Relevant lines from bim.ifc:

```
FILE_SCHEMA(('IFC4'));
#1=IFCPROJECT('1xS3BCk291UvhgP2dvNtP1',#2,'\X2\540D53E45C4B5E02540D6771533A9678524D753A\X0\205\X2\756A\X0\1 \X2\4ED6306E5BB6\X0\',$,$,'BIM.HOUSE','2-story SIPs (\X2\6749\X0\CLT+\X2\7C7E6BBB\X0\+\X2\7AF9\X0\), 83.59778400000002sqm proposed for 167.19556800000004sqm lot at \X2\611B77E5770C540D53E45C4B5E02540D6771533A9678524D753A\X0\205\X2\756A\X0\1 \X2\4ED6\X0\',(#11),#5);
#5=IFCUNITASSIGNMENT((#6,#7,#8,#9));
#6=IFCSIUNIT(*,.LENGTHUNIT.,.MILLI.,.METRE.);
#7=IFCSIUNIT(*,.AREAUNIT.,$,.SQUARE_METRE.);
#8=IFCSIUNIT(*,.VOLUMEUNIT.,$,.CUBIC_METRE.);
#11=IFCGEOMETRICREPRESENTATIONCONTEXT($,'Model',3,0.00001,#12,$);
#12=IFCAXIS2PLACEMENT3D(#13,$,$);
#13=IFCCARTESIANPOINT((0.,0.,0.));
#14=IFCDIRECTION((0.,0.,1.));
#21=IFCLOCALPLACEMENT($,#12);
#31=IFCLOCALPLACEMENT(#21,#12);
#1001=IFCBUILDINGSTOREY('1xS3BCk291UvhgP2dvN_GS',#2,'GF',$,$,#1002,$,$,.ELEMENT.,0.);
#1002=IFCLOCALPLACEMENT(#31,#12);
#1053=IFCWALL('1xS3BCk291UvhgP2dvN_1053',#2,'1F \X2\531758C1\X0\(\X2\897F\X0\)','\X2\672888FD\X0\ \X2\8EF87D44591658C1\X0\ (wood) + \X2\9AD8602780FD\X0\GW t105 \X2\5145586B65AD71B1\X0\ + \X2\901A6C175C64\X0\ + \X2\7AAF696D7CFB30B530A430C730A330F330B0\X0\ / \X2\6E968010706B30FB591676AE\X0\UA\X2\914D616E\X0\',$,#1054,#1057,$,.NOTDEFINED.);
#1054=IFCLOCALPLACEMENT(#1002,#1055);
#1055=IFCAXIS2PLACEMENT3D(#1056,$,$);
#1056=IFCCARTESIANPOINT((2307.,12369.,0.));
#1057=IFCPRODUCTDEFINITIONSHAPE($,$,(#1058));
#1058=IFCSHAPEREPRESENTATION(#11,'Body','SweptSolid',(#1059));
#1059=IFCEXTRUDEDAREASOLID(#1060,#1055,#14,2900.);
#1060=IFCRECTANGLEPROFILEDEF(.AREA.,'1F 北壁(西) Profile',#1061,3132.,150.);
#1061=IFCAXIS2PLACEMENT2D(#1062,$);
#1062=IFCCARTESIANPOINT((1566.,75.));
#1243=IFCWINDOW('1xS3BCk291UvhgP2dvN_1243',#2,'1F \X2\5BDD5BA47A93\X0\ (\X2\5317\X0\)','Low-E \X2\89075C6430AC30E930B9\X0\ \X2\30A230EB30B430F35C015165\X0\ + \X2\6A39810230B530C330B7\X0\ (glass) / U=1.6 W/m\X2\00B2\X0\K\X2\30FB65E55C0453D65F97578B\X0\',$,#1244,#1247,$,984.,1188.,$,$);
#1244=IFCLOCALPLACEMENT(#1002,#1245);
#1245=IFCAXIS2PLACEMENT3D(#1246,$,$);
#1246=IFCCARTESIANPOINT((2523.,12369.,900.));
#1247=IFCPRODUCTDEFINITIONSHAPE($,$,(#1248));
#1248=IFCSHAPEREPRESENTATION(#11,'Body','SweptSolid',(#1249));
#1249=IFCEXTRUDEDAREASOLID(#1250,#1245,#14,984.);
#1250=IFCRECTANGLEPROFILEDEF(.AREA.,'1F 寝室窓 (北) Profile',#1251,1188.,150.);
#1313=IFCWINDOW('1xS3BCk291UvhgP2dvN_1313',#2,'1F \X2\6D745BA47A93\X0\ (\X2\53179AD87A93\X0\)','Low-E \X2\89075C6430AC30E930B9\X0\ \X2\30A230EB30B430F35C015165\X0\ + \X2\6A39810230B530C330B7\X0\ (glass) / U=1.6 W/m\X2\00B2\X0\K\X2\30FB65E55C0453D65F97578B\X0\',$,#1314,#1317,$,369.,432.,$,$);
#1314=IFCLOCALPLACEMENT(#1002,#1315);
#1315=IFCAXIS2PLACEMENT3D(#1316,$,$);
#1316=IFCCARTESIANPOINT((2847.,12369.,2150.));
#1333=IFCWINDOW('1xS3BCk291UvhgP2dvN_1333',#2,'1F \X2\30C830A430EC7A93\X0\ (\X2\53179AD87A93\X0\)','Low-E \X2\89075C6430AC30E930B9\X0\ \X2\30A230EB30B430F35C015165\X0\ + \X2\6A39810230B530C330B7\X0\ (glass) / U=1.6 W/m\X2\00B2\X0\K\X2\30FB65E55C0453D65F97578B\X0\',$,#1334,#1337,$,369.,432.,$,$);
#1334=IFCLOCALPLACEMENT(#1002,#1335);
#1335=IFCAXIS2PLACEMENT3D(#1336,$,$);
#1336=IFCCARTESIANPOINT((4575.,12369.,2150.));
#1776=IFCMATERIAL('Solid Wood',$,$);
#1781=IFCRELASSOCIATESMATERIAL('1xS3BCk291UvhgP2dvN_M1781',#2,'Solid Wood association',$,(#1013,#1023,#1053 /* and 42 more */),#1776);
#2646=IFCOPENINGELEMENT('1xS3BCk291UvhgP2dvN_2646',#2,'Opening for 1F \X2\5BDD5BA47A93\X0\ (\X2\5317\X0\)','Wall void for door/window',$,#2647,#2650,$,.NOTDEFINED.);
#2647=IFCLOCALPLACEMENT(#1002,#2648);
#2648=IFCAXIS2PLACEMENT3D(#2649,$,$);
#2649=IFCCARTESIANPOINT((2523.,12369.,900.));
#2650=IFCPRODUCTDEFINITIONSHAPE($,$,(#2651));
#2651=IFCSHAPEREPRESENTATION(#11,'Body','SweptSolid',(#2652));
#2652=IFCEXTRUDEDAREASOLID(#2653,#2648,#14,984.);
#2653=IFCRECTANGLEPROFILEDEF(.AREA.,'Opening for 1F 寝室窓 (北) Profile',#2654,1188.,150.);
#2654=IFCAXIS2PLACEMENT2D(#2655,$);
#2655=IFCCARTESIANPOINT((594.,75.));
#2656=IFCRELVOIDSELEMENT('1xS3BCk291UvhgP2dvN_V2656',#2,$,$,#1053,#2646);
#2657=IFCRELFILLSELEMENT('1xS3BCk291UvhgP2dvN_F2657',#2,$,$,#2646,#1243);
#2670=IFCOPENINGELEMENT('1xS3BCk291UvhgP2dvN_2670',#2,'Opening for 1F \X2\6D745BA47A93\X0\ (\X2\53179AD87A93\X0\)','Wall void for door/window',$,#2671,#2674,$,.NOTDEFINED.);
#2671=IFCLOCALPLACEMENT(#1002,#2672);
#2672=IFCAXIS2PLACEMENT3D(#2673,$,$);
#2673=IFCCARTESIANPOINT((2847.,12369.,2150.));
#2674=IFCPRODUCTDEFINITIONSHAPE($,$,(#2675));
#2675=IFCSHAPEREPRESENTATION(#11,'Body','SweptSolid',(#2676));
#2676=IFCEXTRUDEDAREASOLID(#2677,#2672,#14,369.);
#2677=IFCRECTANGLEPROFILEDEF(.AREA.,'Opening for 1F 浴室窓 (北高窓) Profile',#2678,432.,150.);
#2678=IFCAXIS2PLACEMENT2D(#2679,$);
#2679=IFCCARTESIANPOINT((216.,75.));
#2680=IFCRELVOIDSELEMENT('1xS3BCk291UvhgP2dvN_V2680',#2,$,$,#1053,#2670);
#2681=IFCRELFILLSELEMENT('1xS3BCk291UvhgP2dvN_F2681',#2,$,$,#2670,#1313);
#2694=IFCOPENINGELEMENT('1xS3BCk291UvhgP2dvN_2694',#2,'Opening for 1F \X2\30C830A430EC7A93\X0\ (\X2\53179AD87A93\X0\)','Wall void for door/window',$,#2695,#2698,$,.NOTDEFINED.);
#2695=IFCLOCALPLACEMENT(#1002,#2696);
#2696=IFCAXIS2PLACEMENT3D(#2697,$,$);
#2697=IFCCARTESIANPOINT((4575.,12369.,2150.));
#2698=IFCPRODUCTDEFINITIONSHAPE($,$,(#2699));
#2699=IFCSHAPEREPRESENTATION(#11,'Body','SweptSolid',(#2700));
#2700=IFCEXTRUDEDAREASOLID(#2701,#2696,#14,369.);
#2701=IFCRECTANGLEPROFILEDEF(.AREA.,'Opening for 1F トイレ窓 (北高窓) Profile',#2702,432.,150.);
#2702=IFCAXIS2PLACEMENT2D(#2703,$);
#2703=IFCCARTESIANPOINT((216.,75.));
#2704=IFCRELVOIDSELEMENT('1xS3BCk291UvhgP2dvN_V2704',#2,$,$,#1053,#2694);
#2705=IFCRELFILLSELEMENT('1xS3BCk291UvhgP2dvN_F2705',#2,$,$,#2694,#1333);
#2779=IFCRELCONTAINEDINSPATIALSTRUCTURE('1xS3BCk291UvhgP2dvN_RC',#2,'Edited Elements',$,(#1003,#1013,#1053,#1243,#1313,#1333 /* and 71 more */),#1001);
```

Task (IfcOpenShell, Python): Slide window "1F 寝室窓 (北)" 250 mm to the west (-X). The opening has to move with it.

```python
import ifcopenshell
import ifcopenshell.api.geometry
import ifcopenshell.util.placement
import ifcopenshell.util.unit

model = ifcopenshell.open("bim.ifc")
unit_scale = ifcopenshell.util.unit.calculate_unit_scale(model)

window = model.by_guid("1xS3BCk291UvhgP2dvN_1243")
opening = window.FillsVoids[0].RelatingOpeningElement
wall = opening.VoidsElements[0].RelatingBuildingElement

wall_matrix = ifcopenshell.util.placement.get_local_placement(wall.ObjectPlacement)
shift = wall_matrix[:3, 0] * -0.25 / unit_scale
before = ifcopenshell.util.placement.get_local_placement(window.ObjectPlacement)[:3, 3].copy()

# The window is not placed relative to its opening, so move both.
for product in (opening, window):
    matrix = ifcopenshell.util.placement.get_local_placement(product.ObjectPlacement)
    matrix[:3, 3] += shift
    ifcopenshell.api.geometry.edit_object_placement(model, product=product, matrix=matrix, is_si=False)

after = ifcopenshell.util.placement.get_local_placement(window.ObjectPlacement)[:3, 3]
print("window moved by", (after - before).round(3) + 0.0)

model.write("bim_updated.ifc")
```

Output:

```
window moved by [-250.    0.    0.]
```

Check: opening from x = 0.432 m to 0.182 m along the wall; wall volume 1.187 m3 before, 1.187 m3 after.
